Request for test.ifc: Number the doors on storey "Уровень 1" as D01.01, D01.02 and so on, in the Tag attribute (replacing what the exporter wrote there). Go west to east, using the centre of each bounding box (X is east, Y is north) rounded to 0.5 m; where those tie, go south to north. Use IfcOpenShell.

First a look at what the model holds.

```python
import ifcopenshell
import ifcopenshell.util.element
import ifcopenshell.util.placement

model = ifcopenshell.open("test.ifc")
print(model.schema)
storey = next(s for s in model.by_type("IfcBuildingStorey") if s.Name == "Уровень 1")
doors = [e for e in ifcopenshell.util.element.get_decomposition(storey) if e.is_a("IfcDoor")]
for e in sorted(doors, key=lambda e: e.id()):
    origin = ifcopenshell.util.placement.get_local_placement(e.ObjectPlacement)[:3, 3]
    print(e.id(), e.Tag, e.Name, origin.round(2) + 0.0, sep=" | ")
```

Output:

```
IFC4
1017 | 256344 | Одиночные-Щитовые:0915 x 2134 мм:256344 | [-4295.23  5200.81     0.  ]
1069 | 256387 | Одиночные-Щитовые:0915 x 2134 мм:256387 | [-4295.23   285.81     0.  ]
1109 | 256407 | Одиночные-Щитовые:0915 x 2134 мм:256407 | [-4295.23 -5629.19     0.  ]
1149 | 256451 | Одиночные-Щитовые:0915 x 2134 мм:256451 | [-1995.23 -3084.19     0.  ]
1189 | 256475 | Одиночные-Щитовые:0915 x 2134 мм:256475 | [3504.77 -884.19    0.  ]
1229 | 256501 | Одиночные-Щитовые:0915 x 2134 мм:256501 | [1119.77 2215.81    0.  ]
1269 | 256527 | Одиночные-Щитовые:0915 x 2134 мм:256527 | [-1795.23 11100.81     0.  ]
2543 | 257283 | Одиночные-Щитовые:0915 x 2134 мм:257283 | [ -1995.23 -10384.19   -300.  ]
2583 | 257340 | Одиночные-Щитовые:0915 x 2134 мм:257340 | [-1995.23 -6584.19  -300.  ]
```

```python
import ifcopenshell
import ifcopenshell.geom
import ifcopenshell.util.element
import ifcopenshell.util.shape

model = ifcopenshell.open("test.ifc")
settings = ifcopenshell.geom.settings()
settings.set("use-world-coords", True)


def centre(element):
    shape = ifcopenshell.geom.create_shape(settings, element)
    return ifcopenshell.util.shape.get_bbox_centroid(shape.geometry)


storey = next(s for s in model.by_type("IfcBuildingStorey") if s.Name == "Уровень 1")
doors = [e for e in ifcopenshell.util.element.get_decomposition(storey) if e.is_a("IfcDoor")]

# Insertion points can sit at a corner or the storey origin, so sort by the geometry (in metres).
centres = {e: centre(e) for e in doors}
doors.sort(key=lambda e: (round(centres[e][0] / 0.5), centres[e][1]))

for i, e in enumerate(doors, start=1):
    number = f"D01.{i:02d}"
    e.Tag = number
    print(e.id(), number)

model.write("test_v2.ifc")
```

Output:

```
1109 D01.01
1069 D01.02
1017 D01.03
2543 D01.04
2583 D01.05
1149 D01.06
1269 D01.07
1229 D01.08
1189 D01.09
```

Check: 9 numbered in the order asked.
